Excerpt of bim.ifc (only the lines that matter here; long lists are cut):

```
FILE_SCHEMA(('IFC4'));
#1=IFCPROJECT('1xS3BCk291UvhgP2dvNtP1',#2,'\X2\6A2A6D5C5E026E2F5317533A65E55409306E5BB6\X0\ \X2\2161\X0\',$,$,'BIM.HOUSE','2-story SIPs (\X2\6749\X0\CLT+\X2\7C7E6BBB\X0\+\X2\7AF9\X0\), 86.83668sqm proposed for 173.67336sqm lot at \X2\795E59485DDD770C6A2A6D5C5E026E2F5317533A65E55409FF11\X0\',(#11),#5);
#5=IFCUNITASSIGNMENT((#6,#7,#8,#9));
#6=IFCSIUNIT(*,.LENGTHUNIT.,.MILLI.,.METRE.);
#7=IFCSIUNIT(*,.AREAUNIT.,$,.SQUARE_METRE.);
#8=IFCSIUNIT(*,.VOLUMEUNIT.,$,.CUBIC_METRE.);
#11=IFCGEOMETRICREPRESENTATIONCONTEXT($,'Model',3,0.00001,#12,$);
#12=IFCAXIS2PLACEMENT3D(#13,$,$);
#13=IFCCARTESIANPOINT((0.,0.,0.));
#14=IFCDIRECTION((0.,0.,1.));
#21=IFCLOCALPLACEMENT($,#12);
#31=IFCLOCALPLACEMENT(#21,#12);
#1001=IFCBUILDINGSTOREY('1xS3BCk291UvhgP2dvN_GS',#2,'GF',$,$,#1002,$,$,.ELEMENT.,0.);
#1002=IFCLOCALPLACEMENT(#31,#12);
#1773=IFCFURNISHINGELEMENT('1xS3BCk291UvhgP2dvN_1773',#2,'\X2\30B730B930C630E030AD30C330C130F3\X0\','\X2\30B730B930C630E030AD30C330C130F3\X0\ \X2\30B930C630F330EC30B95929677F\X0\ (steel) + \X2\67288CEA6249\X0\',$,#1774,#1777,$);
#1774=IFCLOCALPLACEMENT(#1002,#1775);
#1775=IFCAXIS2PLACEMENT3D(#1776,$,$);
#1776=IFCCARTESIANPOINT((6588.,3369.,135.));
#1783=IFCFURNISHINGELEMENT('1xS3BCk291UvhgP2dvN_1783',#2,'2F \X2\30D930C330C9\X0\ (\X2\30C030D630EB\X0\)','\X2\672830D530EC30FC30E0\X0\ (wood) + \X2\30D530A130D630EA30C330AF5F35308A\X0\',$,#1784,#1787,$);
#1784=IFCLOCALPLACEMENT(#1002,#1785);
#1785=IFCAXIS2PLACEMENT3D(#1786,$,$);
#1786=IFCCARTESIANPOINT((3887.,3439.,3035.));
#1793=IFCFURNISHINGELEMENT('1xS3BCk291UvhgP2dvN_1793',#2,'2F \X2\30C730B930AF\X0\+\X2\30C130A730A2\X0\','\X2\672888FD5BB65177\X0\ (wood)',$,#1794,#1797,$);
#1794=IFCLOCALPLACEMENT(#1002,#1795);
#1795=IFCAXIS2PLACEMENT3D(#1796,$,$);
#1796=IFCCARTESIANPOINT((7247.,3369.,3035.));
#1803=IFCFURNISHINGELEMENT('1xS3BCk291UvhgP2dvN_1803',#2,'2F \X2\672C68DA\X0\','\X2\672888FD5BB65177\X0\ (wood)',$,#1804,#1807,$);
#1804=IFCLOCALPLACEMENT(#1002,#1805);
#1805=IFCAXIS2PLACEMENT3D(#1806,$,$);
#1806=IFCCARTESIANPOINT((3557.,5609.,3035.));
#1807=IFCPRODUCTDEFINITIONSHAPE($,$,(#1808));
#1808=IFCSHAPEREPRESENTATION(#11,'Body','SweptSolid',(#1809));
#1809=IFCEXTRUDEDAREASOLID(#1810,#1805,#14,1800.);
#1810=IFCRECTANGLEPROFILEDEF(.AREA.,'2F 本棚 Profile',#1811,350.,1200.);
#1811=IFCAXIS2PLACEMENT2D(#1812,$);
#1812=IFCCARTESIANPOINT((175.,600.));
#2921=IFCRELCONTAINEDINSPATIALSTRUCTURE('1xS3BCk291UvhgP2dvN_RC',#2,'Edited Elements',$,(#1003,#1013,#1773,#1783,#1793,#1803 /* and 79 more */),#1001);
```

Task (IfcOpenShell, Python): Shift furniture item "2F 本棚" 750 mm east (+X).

```python
import ifcopenshell
import ifcopenshell.api.geometry
import ifcopenshell.util.placement
import ifcopenshell.util.unit

model = ifcopenshell.open("bim.ifc")
unit_scale = ifcopenshell.util.unit.calculate_unit_scale(model)

item = model.by_id(1803)
matrix = ifcopenshell.util.placement.get_local_placement(item.ObjectPlacement)
matrix[0, 3] += 0.75 / unit_scale
ifcopenshell.api.geometry.edit_object_placement(model, product=item, matrix=matrix, is_si=False)

print(ifcopenshell.util.placement.get_local_placement(item.ObjectPlacement).round(3) + 0.0)

model.write("bim_rev.ifc")
```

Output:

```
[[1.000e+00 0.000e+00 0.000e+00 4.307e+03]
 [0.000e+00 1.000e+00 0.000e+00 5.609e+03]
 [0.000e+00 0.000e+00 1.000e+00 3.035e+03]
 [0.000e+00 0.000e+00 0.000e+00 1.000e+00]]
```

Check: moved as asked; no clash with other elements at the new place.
